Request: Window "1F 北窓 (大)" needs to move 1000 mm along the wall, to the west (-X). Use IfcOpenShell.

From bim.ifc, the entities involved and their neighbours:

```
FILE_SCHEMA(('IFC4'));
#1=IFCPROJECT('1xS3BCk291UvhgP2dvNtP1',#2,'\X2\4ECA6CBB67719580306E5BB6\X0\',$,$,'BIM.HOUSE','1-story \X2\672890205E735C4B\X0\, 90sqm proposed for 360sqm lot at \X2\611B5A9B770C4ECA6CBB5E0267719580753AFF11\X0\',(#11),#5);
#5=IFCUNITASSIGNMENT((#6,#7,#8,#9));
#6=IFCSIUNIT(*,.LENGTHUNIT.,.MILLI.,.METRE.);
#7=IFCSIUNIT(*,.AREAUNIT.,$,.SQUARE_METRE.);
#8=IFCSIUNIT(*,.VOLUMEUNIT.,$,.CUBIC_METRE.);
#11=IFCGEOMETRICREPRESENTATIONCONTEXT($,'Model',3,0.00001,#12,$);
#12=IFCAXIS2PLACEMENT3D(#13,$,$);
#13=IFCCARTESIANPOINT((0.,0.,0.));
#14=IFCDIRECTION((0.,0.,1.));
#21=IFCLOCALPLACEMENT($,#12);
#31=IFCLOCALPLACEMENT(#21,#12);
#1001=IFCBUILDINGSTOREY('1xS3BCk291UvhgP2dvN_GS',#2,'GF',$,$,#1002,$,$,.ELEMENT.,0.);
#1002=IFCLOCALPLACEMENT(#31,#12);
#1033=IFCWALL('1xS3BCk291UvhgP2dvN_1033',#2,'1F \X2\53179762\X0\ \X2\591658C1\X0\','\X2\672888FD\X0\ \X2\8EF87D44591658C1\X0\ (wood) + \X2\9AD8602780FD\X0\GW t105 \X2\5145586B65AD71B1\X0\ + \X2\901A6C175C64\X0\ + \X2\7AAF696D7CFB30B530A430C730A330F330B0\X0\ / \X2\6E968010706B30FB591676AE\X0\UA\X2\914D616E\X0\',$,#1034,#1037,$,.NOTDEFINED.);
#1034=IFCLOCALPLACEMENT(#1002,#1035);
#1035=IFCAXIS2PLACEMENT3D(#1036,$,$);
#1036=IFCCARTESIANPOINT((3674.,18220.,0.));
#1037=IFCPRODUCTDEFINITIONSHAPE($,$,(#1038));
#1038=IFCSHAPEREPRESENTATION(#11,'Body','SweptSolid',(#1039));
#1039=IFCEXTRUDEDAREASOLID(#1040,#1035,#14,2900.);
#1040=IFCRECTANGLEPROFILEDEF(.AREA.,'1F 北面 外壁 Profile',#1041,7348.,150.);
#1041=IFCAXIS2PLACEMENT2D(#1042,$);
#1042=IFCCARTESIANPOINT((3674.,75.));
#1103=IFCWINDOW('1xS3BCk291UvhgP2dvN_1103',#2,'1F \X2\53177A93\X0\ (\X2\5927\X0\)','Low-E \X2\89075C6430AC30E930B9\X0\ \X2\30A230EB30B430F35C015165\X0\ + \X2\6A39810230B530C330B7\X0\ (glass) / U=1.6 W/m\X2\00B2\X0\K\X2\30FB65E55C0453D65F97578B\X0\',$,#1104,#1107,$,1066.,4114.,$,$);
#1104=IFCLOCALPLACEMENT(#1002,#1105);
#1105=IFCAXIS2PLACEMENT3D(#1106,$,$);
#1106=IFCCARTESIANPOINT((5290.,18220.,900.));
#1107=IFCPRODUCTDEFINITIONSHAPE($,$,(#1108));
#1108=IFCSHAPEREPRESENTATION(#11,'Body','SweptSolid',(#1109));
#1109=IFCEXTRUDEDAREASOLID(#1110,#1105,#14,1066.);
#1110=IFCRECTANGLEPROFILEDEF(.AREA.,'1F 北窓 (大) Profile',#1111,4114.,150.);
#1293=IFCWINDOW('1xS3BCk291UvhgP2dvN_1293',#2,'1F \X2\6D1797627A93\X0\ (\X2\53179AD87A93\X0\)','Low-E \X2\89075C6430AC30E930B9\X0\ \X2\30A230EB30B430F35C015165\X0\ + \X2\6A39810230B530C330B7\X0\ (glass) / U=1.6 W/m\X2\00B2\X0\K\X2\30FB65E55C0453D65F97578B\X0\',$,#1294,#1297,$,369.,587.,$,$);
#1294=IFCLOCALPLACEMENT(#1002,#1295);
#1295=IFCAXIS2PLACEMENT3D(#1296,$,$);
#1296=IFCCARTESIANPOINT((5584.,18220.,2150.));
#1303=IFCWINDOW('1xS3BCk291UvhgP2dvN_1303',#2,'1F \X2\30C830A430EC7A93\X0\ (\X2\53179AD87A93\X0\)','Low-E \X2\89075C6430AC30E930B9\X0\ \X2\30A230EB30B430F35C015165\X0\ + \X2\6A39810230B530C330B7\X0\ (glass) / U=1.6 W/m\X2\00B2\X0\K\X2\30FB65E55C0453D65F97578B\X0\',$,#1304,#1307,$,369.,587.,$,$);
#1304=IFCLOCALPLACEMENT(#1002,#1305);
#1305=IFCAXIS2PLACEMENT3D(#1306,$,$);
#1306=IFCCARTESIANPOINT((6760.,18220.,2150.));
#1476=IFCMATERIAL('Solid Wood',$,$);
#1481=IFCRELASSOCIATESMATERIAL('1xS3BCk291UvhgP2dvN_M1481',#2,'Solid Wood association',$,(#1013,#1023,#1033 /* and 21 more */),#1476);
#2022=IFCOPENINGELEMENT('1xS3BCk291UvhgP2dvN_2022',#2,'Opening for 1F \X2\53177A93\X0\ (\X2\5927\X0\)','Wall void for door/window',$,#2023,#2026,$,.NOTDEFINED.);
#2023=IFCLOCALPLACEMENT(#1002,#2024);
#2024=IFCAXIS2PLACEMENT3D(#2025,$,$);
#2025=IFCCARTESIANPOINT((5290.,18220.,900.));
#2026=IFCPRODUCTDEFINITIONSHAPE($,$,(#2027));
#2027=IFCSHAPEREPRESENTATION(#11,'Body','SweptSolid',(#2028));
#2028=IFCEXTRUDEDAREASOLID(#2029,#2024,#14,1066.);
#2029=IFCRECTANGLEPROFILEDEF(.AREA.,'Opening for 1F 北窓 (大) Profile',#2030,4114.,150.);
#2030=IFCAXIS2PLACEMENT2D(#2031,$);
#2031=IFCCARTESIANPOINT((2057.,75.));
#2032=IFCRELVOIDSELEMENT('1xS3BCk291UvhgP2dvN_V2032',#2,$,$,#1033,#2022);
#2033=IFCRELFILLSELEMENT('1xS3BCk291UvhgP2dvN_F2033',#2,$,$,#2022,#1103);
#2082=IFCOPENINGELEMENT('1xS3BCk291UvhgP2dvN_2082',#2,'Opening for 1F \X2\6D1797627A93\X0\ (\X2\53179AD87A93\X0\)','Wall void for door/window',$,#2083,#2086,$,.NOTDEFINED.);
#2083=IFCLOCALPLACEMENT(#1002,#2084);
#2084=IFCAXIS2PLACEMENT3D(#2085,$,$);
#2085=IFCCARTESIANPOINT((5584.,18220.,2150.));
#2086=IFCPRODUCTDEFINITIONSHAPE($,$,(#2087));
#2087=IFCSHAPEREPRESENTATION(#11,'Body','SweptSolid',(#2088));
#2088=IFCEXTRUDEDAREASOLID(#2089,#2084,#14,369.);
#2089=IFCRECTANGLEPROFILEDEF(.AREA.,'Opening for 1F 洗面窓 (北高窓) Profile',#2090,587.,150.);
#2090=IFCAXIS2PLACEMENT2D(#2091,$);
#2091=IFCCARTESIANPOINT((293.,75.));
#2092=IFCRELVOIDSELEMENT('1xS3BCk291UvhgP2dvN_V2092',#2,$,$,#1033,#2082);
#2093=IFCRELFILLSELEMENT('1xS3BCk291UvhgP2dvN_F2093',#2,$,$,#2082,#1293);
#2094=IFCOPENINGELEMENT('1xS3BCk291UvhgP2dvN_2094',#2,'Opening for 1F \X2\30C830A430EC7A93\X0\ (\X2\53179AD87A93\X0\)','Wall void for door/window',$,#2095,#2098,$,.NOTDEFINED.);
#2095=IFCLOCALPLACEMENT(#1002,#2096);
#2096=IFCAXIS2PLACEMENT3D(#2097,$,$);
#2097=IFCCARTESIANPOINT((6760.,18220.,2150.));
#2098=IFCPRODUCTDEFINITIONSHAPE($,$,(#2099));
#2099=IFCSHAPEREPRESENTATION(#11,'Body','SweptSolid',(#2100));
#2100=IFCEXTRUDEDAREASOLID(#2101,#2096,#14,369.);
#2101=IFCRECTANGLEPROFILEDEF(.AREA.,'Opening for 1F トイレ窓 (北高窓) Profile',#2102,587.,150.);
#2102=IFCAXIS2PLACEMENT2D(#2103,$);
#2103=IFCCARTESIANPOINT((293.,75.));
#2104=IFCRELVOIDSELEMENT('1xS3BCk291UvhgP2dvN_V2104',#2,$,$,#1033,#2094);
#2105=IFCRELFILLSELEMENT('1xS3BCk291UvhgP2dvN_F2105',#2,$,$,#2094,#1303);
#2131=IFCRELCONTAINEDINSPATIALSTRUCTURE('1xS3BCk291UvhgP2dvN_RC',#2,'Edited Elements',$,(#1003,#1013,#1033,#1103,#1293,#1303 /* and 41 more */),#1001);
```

```python
import ifcopenshell
import ifcopenshell.api.geometry
import ifcopenshell.util.placement

model = ifcopenshell.open("bim.ifc")

window = model.by_guid("1xS3BCk291UvhgP2dvN_1103")
opening = window.FillsVoids[0].RelatingOpeningElement
wall = opening.VoidsElements[0].RelatingBuildingElement

wall_matrix = ifcopenshell.util.placement.get_local_placement(wall.ObjectPlacement)
shift = wall_matrix[:3, 0] * -1000.0
before = ifcopenshell.util.placement.get_local_placement(window.ObjectPlacement)[:3, 3].copy()

# The window is not placed relative to its opening, so move both.
for product in (opening, window):
    matrix = ifcopenshell.util.placement.get_local_placement(product.ObjectPlacement)
    matrix[:3, 3] += shift
    ifcopenshell.api.geometry.edit_object_placement(model, product=product, matrix=matrix, is_si=False)

after = ifcopenshell.util.placement.get_local_placement(window.ObjectPlacement)[:3, 3]
print("window moved by", (after - before).round(3) + 0.0)

model.write("bim_v2.ifc")
```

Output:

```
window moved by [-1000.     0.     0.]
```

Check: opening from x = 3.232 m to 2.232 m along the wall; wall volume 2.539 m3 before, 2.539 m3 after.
